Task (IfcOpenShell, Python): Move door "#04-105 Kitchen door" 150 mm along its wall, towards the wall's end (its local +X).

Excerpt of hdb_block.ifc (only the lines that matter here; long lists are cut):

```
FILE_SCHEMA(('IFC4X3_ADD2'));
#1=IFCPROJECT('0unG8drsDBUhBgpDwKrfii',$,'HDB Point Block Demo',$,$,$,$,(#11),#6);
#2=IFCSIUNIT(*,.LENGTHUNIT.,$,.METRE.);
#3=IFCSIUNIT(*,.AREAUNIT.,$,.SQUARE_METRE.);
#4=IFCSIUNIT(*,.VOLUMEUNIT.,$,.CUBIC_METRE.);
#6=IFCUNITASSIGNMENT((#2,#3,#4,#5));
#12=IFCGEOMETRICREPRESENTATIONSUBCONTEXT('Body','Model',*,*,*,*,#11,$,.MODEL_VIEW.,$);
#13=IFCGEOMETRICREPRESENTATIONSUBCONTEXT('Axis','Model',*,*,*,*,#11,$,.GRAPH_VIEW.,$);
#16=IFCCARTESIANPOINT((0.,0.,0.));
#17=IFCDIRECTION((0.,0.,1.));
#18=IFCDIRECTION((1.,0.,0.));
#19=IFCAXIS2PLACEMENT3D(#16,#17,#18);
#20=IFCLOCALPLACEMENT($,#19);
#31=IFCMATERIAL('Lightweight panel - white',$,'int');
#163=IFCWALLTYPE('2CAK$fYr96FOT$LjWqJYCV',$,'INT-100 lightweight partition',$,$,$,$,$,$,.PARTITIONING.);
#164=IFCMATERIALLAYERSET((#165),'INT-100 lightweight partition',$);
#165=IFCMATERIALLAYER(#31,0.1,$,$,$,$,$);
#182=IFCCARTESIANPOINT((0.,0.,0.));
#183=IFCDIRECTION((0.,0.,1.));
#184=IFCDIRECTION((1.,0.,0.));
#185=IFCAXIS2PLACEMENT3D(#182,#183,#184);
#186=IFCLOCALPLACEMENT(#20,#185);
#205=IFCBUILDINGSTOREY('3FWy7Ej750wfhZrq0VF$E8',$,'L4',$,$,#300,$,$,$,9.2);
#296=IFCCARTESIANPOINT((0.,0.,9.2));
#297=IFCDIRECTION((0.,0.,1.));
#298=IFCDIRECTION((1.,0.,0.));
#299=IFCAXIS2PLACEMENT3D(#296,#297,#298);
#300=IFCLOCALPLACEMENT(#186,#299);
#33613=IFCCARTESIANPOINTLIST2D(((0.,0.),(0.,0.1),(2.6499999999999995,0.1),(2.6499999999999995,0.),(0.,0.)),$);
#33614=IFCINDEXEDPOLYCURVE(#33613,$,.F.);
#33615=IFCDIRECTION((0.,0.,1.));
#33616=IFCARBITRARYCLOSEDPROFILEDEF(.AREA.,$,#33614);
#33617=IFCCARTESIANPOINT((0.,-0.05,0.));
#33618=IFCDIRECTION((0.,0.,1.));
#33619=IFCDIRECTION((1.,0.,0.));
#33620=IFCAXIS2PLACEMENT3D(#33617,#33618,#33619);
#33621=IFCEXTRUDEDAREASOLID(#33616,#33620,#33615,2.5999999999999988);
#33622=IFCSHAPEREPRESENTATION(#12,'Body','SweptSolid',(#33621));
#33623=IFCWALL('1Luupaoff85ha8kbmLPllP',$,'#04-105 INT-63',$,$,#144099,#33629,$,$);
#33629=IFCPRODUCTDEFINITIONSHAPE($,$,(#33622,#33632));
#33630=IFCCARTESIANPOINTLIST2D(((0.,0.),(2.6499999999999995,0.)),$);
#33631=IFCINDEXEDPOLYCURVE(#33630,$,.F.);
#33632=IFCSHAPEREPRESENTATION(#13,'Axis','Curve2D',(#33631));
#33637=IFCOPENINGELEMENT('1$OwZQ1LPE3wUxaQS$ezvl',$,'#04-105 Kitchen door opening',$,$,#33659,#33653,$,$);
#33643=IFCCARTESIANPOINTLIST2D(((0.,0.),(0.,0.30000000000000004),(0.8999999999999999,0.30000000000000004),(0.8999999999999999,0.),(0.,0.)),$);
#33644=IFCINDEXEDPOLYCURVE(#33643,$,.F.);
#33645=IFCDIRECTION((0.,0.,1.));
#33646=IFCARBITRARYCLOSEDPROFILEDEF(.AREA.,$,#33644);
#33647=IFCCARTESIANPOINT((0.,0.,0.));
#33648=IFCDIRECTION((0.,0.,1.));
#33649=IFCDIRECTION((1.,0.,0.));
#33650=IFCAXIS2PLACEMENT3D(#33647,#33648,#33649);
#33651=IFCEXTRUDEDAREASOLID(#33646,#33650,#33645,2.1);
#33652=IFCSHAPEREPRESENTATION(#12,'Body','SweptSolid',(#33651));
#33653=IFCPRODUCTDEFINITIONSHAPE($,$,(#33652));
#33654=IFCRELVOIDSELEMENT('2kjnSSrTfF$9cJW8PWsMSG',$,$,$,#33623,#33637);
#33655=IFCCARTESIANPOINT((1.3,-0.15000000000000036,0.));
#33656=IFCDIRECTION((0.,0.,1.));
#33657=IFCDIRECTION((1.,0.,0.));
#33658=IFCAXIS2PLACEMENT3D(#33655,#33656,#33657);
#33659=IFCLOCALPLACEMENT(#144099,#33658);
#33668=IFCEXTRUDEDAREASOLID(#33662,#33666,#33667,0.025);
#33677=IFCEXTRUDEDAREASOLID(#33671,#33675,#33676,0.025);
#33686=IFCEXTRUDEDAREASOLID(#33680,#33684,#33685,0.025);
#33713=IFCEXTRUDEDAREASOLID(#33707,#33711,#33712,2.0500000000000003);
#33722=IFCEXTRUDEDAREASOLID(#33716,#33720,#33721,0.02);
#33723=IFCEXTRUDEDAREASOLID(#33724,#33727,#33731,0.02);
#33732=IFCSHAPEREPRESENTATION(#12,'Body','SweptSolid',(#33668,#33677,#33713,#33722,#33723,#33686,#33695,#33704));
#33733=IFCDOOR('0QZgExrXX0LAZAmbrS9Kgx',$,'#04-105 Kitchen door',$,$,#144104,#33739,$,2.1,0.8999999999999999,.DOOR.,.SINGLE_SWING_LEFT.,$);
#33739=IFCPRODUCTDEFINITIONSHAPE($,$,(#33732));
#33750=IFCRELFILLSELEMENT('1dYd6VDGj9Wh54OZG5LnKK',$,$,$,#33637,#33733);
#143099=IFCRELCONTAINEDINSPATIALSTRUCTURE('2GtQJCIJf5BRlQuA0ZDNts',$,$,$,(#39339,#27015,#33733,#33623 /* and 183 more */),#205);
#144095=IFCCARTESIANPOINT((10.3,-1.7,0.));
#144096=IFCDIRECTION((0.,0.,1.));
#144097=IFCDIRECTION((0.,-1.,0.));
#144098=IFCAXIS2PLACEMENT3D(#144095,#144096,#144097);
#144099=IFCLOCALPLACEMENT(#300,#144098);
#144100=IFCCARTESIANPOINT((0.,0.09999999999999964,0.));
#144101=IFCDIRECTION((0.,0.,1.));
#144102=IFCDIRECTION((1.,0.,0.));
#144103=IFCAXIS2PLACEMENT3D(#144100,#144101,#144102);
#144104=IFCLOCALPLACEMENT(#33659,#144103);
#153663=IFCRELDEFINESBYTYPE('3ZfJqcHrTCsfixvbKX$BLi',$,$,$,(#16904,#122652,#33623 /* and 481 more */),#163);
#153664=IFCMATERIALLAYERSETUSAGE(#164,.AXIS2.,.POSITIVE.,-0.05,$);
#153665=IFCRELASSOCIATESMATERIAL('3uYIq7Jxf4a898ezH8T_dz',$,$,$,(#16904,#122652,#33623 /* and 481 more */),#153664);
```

```python
import ifcopenshell
import ifcopenshell.api.geometry
import ifcopenshell.util.placement

model = ifcopenshell.open("hdb_block.ifc")

door = model.by_guid("0QZgExrXX0LAZAmbrS9Kgx")
opening = door.FillsVoids[0].RelatingOpeningElement
wall = opening.VoidsElements[0].RelatingBuildingElement

wall_matrix = ifcopenshell.util.placement.get_local_placement(wall.ObjectPlacement)
shift = wall_matrix[:3, 0] * 0.15
before = ifcopenshell.util.placement.get_local_placement(door.ObjectPlacement)[:3, 3].copy()

# The door is placed relative to its opening, so it follows when the opening moves.
matrix = ifcopenshell.util.placement.get_local_placement(opening.ObjectPlacement)
matrix[:3, 3] += shift
ifcopenshell.api.geometry.edit_object_placement(
    model, product=opening, matrix=matrix, is_si=False, should_transform_children=True
)

after = ifcopenshell.util.placement.get_local_placement(door.ObjectPlacement)[:3, 3]
print("door moved by", (after - before).round(3) + 0.0)

model.write("hdb_block_updated.ifc")
```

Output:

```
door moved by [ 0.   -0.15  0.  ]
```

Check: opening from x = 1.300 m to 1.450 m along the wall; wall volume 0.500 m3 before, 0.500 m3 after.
